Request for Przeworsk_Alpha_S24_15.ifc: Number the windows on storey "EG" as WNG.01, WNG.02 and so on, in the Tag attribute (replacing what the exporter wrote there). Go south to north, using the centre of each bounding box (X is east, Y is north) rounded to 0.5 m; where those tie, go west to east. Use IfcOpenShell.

First a look at what the model holds.

```python
import ifcopenshell
import ifcopenshell.util.element
import ifcopenshell.util.placement

model = ifcopenshell.open("Przeworsk_Alpha_S24_15.ifc")
print(model.schema)
storey = next(s for s in model.by_type("IfcBuildingStorey") if s.Name == "EG")
windows = [e for e in ifcopenshell.util.element.get_decomposition(storey) if e.is_a("IfcWindow")]
for e in sorted(windows, key=lambda e: e.id()):
    origin = ifcopenshell.util.placement.get_local_placement(e.ObjectPlacement)[:3, 3]
    print(e.id(), e.Tag, e.Name, origin.round(2) + 0.0, sep=" | ")
```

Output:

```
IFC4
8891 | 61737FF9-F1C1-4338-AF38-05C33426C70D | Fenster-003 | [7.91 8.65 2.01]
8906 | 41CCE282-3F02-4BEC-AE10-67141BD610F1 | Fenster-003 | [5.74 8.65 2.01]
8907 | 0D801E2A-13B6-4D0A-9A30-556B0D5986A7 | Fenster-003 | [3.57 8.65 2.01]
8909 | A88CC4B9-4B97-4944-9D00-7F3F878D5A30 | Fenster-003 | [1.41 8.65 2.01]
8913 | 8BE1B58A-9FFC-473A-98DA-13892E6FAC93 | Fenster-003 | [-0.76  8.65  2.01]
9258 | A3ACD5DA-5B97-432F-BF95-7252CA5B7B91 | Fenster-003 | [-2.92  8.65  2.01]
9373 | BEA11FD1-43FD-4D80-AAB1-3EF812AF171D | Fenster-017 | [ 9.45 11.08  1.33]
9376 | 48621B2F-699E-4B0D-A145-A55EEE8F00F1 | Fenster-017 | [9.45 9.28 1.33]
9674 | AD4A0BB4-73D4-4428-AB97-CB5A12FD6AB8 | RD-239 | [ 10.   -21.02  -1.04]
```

```python
import ifcopenshell
import ifcopenshell.geom
import ifcopenshell.util.element
import ifcopenshell.util.shape

model = ifcopenshell.open("Przeworsk_Alpha_S24_15.ifc")
settings = ifcopenshell.geom.settings()
settings.set("use-world-coords", True)


def centre(element):
    shape = ifcopenshell.geom.create_shape(settings, element)
    return ifcopenshell.util.shape.get_bbox_centroid(shape.geometry)


storey = next(s for s in model.by_type("IfcBuildingStorey") if s.Name == "EG")
windows = [e for e in ifcopenshell.util.element.get_decomposition(storey) if e.is_a("IfcWindow")]

# Insertion points can sit at a corner or the storey origin, so sort by the geometry (in metres).
centres = {e: centre(e) for e in windows}
windows.sort(key=lambda e: (round(centres[e][1] / 0.5), centres[e][0]))

for i, e in enumerate(windows, start=1):
    number = f"WNG.{i:02d}"
    e.Tag = number
    print(e.id(), number)

model.write("Przeworsk_Alpha_S24_15_edited.ifc")
```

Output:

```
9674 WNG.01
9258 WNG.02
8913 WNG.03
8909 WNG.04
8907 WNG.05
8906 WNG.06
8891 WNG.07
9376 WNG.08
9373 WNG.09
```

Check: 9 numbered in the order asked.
